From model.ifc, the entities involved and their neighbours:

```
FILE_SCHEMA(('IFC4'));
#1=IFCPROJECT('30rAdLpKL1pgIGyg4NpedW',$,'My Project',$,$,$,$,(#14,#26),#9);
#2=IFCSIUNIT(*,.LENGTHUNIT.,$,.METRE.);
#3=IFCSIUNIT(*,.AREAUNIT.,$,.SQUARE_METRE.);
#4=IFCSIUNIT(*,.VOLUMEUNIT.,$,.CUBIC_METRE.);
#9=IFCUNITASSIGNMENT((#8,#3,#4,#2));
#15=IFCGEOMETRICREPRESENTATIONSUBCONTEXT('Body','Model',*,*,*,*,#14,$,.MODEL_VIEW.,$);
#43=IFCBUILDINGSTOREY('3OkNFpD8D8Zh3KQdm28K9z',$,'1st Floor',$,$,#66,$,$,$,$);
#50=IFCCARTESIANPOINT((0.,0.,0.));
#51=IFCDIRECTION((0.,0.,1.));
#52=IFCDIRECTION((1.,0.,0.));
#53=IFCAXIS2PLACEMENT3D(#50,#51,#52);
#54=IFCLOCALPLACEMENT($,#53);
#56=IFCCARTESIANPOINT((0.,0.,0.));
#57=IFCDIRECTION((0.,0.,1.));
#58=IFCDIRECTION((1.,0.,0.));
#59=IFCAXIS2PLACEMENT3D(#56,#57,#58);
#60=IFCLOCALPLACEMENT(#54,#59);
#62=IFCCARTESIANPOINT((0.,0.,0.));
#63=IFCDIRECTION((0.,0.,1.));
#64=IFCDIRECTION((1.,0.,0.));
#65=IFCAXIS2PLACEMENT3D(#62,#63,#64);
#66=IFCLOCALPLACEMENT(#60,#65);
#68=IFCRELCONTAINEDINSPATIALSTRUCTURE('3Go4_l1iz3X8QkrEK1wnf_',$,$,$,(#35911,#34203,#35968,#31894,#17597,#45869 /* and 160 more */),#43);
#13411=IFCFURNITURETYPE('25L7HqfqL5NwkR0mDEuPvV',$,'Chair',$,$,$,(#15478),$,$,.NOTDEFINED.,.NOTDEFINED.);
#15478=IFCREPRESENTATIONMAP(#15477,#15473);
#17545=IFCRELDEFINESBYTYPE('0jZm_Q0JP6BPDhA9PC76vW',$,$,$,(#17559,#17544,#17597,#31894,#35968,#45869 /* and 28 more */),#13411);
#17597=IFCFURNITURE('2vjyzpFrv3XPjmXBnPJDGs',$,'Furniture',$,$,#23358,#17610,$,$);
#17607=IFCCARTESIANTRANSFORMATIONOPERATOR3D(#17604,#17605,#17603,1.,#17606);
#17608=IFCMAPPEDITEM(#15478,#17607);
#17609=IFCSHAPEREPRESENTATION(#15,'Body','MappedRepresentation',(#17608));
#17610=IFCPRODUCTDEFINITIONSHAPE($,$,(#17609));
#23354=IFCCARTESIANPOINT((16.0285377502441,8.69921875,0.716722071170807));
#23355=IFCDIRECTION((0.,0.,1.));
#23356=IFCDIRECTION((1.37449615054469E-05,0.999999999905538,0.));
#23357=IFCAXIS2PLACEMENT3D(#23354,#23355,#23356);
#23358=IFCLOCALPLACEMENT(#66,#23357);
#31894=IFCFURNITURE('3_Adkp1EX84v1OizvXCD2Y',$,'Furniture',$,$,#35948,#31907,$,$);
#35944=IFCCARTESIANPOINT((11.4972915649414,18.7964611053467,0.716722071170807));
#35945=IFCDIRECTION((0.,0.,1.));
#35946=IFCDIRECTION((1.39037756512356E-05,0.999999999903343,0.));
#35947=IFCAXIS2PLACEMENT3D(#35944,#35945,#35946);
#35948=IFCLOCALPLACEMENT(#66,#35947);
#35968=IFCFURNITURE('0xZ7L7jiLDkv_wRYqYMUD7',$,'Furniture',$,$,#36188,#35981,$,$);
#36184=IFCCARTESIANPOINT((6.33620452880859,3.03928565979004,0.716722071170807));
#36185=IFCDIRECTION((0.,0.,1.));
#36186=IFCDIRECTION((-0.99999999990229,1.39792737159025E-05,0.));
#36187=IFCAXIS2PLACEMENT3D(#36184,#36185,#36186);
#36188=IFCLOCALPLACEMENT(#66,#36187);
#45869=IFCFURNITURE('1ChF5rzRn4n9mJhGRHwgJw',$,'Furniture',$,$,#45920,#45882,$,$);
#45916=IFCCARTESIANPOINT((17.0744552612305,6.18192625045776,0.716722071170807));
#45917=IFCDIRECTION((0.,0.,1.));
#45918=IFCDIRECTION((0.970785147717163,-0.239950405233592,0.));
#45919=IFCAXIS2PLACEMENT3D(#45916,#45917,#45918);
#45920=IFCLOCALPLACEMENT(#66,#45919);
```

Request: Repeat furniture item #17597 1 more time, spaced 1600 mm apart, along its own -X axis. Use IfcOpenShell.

```python
import ifcopenshell
import ifcopenshell.api.geometry
import ifcopenshell.api.root
import ifcopenshell.util.element
import ifcopenshell.util.placement

model = ifcopenshell.open("model.ifc")

source = model.by_id(17597)
base = ifcopenshell.util.placement.get_local_placement(source.ObjectPlacement)
step = -base[:3, 0] * 1.6

for i in range(1, 2):
    copy = ifcopenshell.api.root.copy_class(model, product=source)
    copy.Representation = ifcopenshell.util.element.copy_deep(
        model, source.Representation, exclude=["IfcGeometricRepresentationContext", "IfcRepresentationMap"]
    )
    matrix = base.copy()
    matrix[:3, 3] += i * step
    print("added at", matrix[:3, 3].round(3) + 0.0)
    ifcopenshell.api.geometry.edit_object_placement(model, product=copy, matrix=matrix, is_si=False)

model.write("model_v2.ifc")
```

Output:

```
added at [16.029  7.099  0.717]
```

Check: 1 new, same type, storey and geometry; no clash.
